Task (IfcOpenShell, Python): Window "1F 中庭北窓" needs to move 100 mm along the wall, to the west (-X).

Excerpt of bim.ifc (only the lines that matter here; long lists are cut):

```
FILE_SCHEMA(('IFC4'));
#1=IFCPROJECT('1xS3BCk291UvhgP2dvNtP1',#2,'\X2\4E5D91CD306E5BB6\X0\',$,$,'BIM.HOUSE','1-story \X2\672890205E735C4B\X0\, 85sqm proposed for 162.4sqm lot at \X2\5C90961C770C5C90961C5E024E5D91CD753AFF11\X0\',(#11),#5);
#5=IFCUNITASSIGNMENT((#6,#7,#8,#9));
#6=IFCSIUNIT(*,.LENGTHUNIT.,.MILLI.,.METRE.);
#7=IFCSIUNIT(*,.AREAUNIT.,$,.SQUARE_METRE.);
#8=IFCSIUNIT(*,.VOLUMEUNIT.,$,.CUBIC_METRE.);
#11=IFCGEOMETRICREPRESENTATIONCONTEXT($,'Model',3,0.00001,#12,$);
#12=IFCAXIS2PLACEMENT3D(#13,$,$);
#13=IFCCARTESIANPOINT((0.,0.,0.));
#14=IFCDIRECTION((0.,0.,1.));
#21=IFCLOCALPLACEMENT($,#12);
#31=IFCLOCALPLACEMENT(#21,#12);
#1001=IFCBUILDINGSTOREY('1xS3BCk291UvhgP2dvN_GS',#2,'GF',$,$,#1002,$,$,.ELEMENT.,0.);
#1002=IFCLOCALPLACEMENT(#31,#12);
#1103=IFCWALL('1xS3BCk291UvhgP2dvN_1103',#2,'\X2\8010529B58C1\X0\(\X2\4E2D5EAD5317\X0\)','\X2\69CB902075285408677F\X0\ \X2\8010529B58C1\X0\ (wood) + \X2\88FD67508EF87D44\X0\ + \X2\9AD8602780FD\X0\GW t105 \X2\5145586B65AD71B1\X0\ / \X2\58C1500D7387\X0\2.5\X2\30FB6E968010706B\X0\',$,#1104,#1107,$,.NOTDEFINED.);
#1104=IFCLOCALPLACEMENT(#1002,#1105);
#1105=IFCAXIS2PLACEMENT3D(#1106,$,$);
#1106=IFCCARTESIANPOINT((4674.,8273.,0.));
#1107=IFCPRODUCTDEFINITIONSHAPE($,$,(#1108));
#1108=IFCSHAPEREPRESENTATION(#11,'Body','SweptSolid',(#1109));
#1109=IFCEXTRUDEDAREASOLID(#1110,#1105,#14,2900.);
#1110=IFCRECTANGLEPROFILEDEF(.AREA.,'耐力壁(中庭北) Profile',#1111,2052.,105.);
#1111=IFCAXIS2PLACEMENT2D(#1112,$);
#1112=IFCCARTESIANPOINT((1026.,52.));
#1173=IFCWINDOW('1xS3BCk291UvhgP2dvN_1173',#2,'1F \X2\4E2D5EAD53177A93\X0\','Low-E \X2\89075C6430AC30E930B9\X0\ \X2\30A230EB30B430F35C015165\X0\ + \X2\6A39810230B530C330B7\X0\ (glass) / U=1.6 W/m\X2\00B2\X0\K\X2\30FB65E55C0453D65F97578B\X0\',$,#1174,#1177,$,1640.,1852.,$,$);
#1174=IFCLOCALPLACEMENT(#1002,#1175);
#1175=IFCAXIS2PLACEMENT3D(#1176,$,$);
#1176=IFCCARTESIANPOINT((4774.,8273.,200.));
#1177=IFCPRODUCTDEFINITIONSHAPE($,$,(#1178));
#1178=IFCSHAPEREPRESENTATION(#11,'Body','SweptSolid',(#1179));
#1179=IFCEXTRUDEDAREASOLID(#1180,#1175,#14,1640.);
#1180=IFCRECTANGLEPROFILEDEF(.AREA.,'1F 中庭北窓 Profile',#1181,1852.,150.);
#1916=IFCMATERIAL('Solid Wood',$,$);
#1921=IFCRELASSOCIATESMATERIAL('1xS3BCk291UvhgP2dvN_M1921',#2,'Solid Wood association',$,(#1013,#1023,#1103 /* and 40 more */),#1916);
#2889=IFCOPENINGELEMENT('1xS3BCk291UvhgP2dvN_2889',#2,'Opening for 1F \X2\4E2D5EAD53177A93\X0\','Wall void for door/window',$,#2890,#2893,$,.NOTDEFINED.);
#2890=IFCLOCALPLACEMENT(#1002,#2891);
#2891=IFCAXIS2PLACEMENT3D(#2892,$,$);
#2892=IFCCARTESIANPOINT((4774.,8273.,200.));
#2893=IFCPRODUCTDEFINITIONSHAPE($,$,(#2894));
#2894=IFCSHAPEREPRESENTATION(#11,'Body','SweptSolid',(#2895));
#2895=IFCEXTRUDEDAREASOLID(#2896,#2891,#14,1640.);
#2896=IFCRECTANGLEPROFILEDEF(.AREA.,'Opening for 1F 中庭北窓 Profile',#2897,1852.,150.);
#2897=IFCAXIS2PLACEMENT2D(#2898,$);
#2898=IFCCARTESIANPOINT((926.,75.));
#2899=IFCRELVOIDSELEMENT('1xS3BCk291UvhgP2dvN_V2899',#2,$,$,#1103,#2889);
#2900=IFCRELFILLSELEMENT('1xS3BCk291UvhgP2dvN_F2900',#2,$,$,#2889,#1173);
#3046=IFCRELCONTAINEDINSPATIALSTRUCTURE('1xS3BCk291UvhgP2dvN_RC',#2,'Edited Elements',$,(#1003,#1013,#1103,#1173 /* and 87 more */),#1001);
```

```python
import ifcopenshell
import ifcopenshell.api.geometry
import ifcopenshell.util.placement
import ifcopenshell.util.unit

model = ifcopenshell.open("bim.ifc")
unit_scale = ifcopenshell.util.unit.calculate_unit_scale(model)

window = model.by_guid("1xS3BCk291UvhgP2dvN_1173")
opening = window.FillsVoids[0].RelatingOpeningElement
wall = opening.VoidsElements[0].RelatingBuildingElement

wall_matrix = ifcopenshell.util.placement.get_local_placement(wall.ObjectPlacement)
shift = wall_matrix[:3, 0] * -0.1 / unit_scale
before = ifcopenshell.util.placement.get_local_placement(window.ObjectPlacement)[:3, 3].copy()

# The window is not placed relative to its opening, so move both.
for product in (opening, window):
    matrix = ifcopenshell.util.placement.get_local_placement(product.ObjectPlacement)
    matrix[:3, 3] += shift
    ifcopenshell.api.geometry.edit_object_placement(model, product=product, matrix=matrix, is_si=False)

after = ifcopenshell.util.placement.get_local_placement(window.ObjectPlacement)[:3, 3]
print("window moved by", (after - before).round(3) + 0.0)

model.write("bim_updated.ifc")
```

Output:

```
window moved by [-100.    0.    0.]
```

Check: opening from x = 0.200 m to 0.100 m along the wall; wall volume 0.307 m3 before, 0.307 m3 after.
